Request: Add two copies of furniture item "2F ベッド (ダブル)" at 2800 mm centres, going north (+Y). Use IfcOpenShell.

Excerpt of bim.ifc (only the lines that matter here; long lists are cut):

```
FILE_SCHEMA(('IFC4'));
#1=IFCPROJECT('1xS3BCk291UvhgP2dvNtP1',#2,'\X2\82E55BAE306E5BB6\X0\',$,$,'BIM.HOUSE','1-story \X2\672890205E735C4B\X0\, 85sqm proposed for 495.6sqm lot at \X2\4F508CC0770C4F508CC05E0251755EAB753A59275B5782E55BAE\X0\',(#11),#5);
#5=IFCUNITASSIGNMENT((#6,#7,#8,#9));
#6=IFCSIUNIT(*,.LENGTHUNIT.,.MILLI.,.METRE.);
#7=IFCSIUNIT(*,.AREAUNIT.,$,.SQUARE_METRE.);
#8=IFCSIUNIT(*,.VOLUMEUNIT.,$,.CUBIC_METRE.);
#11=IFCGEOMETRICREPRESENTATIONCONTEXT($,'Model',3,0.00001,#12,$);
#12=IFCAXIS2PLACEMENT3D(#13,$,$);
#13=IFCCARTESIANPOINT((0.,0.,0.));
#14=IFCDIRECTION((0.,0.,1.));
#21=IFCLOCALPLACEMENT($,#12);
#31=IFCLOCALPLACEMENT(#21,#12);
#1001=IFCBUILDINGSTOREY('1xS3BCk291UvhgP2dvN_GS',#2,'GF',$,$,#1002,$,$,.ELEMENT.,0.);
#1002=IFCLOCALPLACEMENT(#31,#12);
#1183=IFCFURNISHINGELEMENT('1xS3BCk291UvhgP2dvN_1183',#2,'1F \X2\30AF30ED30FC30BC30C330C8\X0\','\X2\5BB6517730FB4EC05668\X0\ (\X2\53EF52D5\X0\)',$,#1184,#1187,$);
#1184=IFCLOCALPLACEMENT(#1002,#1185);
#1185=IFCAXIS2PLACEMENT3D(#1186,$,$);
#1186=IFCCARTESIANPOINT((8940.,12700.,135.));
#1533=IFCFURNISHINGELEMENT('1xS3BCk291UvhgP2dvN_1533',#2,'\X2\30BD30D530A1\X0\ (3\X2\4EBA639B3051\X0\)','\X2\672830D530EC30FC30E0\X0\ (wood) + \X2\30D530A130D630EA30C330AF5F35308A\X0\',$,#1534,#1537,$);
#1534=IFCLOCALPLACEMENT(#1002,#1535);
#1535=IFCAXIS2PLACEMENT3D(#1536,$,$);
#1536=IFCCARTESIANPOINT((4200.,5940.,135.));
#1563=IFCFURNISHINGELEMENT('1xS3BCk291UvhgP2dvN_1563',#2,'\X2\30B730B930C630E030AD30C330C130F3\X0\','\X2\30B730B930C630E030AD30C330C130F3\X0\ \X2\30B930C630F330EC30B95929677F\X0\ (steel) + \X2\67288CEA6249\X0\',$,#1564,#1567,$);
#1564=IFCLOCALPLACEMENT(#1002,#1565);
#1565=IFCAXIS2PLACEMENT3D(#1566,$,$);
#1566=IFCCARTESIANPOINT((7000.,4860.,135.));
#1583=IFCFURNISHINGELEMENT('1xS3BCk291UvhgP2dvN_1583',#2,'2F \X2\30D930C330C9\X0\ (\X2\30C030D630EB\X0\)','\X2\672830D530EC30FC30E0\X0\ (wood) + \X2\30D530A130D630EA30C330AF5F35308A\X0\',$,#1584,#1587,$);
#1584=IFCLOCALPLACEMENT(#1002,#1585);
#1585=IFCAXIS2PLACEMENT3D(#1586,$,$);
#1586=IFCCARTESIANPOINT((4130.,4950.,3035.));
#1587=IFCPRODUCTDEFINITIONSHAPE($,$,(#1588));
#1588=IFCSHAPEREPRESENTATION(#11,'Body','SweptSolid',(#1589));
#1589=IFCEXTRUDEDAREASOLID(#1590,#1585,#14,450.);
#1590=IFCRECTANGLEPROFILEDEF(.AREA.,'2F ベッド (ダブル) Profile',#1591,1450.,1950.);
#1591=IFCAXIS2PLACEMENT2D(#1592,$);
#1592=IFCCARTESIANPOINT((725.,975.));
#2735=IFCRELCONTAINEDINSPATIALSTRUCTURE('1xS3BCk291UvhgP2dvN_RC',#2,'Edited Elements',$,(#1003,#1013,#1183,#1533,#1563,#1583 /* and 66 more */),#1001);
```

```python
import numpy as np
import ifcopenshell
import ifcopenshell.api.geometry
import ifcopenshell.api.root
import ifcopenshell.util.element
import ifcopenshell.util.placement

model = ifcopenshell.open("bim.ifc")


def reuse_history(source, copy):
    """copy_class also copies each property set's owner history, people and application; keep the originals."""
    for rel in copy.IsDefinedBy:
        if rel.is_a("IfcRelDefinesByProperties") and (history := rel.RelatingPropertyDefinition.OwnerHistory):
            rel.RelatingPropertyDefinition.OwnerHistory = source.OwnerHistory
            ifcopenshell.util.element.remove_deep2(model, history)


source = model.by_guid("1xS3BCk291UvhgP2dvN_1583")
base = ifcopenshell.util.placement.get_local_placement(source.ObjectPlacement)
step = np.array([0.0, 1.0, 0.0]) * 2800.0

for i in range(1, 3):
    copy = ifcopenshell.api.root.copy_class(model, product=source)
    copy.Representation = ifcopenshell.util.element.copy_deep(
        model, source.Representation, exclude=["IfcGeometricRepresentationContext", "IfcRepresentationMap"]
    )
    reuse_history(source, copy)
    matrix = base.copy()
    matrix[:3, 3] += i * step
    print("added at", matrix[:3, 3].round(3) + 0.0)
    ifcopenshell.api.geometry.edit_object_placement(model, product=copy, matrix=matrix, is_si=False)

model.write("bim_updated.ifc")
```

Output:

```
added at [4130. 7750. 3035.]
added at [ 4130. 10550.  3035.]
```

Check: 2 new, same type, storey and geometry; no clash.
